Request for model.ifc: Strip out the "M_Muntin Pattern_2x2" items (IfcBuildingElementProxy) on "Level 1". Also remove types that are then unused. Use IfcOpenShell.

First a look at what the model holds.

```python
import ifcopenshell
import ifcopenshell.util.element

model = ifcopenshell.open("model.ifc")
print(model.schema)
storey = next(s for s in model.by_type("IfcBuildingStorey") if s.Name == "Level 1")
proxies = [e for e in ifcopenshell.util.element.get_decomposition(storey) if e.is_a("IfcBuildingElementProxy")]
seen = {}
for e in proxies:
    element_type = ifcopenshell.util.element.get_type(e)
    name = element_type.Name if element_type not in (None, e) else None
    seen[name] = seen.get(name, 0) + 1
for name, count in sorted(seen.items(), key=str):
    print(count, "x", name)
```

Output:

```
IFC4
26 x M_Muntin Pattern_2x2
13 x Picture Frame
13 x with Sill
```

```python
import ifcopenshell
import ifcopenshell.api.root
import ifcopenshell.util.element

model = ifcopenshell.open("model.ifc")

storey = next(s for s in model.by_type("IfcBuildingStorey") if s.Name == "Level 1")
proxies = [e for e in ifcopenshell.util.element.get_decomposition(storey) if e.is_a("IfcBuildingElementProxy")]
targets = [e for e in proxies if (t := ifcopenshell.util.element.get_type(e)) not in (None, e) and t.Name == "M_Muntin Pattern_2x2"]
types = {ifcopenshell.util.element.get_type(e) for e in targets} - {None, *targets}

for e in targets:
    ifcopenshell.api.root.remove_product(model, product=e)
print(len(targets), "removed")

unused = [t for t in types if not ifcopenshell.util.element.get_types(t)]
for t in unused:
    ifcopenshell.api.root.remove_product(model, product=t)
print(len(unused), "unused types removed")

model.write("model_rev.ifc")
```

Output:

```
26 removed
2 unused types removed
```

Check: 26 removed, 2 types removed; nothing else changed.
